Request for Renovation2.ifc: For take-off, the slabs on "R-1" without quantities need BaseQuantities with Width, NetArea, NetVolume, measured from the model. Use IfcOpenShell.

First a look at what the model holds.

```python
import ifcopenshell
import ifcopenshell.util.element
import ifcopenshell.util.unit

model = ifcopenshell.open("Renovation2.ifc")
print(model.schema)
for unit_type in ("LENGTHUNIT", "AREAUNIT", "VOLUMEUNIT"):
    print(unit_type, ifcopenshell.util.unit.calculate_unit_scale(model, unit_type))
storey = next(s for s in model.by_type("IfcBuildingStorey") if s.Name == "R-1")
slabs = [e for e in ifcopenshell.util.element.get_decomposition(storey) if e.is_a("IfcSlab")]
for e in sorted(slabs, key=lambda e: e.id()):
    print(e.id(), e.is_a(), e.Name, list(ifcopenshell.util.element.get_psets(e, qtos_only=True)), sep=" | ")
```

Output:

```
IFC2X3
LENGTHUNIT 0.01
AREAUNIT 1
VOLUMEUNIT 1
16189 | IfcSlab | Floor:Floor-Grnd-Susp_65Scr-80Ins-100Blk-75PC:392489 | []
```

```python
import ifcopenshell
import ifcopenshell.api.pset
import ifcopenshell.geom
import ifcopenshell.util.element
import ifcopenshell.util.shape
import ifcopenshell.util.unit

model = ifcopenshell.open("Renovation2.ifc")
unit_scale = ifcopenshell.util.unit.calculate_unit_scale(model)
area_scale = ifcopenshell.util.unit.calculate_unit_scale(model, "AREAUNIT")
volume_scale = ifcopenshell.util.unit.calculate_unit_scale(model, "VOLUMEUNIT")
settings = ifcopenshell.geom.settings()

storey = next(s for s in model.by_type("IfcBuildingStorey") if s.Name == "R-1")
slabs = [e for e in ifcopenshell.util.element.get_decomposition(storey) if e.is_a("IfcSlab")]

for e in sorted(slabs, key=lambda e: e.id()):
    if ifcopenshell.util.element.get_psets(e, qtos_only=True, should_inherit=False):
        continue
    # Geometry comes back in metres, in the element's own axes.
    shape = ifcopenshell.geom.create_shape(settings, e)
    values = {
        "Width": ifcopenshell.util.shape.get_z(shape.geometry) / unit_scale,
        "NetArea": ifcopenshell.util.shape.get_footprint_area(shape.geometry) / area_scale,
        "NetVolume": ifcopenshell.util.shape.get_volume(shape.geometry) / volume_scale,
    }
    qto = ifcopenshell.api.pset.add_qto(model, product=e, name="BaseQuantities")
    ifcopenshell.api.pset.edit_qto(model, qto=qto, properties=values)
    print(e.id(), {k: round(v, 3) for k, v in values.items()})

model.write("Renovation2_v2.ifc")
```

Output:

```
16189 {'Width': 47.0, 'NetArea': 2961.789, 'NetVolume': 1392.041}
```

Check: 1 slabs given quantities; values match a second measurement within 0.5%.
